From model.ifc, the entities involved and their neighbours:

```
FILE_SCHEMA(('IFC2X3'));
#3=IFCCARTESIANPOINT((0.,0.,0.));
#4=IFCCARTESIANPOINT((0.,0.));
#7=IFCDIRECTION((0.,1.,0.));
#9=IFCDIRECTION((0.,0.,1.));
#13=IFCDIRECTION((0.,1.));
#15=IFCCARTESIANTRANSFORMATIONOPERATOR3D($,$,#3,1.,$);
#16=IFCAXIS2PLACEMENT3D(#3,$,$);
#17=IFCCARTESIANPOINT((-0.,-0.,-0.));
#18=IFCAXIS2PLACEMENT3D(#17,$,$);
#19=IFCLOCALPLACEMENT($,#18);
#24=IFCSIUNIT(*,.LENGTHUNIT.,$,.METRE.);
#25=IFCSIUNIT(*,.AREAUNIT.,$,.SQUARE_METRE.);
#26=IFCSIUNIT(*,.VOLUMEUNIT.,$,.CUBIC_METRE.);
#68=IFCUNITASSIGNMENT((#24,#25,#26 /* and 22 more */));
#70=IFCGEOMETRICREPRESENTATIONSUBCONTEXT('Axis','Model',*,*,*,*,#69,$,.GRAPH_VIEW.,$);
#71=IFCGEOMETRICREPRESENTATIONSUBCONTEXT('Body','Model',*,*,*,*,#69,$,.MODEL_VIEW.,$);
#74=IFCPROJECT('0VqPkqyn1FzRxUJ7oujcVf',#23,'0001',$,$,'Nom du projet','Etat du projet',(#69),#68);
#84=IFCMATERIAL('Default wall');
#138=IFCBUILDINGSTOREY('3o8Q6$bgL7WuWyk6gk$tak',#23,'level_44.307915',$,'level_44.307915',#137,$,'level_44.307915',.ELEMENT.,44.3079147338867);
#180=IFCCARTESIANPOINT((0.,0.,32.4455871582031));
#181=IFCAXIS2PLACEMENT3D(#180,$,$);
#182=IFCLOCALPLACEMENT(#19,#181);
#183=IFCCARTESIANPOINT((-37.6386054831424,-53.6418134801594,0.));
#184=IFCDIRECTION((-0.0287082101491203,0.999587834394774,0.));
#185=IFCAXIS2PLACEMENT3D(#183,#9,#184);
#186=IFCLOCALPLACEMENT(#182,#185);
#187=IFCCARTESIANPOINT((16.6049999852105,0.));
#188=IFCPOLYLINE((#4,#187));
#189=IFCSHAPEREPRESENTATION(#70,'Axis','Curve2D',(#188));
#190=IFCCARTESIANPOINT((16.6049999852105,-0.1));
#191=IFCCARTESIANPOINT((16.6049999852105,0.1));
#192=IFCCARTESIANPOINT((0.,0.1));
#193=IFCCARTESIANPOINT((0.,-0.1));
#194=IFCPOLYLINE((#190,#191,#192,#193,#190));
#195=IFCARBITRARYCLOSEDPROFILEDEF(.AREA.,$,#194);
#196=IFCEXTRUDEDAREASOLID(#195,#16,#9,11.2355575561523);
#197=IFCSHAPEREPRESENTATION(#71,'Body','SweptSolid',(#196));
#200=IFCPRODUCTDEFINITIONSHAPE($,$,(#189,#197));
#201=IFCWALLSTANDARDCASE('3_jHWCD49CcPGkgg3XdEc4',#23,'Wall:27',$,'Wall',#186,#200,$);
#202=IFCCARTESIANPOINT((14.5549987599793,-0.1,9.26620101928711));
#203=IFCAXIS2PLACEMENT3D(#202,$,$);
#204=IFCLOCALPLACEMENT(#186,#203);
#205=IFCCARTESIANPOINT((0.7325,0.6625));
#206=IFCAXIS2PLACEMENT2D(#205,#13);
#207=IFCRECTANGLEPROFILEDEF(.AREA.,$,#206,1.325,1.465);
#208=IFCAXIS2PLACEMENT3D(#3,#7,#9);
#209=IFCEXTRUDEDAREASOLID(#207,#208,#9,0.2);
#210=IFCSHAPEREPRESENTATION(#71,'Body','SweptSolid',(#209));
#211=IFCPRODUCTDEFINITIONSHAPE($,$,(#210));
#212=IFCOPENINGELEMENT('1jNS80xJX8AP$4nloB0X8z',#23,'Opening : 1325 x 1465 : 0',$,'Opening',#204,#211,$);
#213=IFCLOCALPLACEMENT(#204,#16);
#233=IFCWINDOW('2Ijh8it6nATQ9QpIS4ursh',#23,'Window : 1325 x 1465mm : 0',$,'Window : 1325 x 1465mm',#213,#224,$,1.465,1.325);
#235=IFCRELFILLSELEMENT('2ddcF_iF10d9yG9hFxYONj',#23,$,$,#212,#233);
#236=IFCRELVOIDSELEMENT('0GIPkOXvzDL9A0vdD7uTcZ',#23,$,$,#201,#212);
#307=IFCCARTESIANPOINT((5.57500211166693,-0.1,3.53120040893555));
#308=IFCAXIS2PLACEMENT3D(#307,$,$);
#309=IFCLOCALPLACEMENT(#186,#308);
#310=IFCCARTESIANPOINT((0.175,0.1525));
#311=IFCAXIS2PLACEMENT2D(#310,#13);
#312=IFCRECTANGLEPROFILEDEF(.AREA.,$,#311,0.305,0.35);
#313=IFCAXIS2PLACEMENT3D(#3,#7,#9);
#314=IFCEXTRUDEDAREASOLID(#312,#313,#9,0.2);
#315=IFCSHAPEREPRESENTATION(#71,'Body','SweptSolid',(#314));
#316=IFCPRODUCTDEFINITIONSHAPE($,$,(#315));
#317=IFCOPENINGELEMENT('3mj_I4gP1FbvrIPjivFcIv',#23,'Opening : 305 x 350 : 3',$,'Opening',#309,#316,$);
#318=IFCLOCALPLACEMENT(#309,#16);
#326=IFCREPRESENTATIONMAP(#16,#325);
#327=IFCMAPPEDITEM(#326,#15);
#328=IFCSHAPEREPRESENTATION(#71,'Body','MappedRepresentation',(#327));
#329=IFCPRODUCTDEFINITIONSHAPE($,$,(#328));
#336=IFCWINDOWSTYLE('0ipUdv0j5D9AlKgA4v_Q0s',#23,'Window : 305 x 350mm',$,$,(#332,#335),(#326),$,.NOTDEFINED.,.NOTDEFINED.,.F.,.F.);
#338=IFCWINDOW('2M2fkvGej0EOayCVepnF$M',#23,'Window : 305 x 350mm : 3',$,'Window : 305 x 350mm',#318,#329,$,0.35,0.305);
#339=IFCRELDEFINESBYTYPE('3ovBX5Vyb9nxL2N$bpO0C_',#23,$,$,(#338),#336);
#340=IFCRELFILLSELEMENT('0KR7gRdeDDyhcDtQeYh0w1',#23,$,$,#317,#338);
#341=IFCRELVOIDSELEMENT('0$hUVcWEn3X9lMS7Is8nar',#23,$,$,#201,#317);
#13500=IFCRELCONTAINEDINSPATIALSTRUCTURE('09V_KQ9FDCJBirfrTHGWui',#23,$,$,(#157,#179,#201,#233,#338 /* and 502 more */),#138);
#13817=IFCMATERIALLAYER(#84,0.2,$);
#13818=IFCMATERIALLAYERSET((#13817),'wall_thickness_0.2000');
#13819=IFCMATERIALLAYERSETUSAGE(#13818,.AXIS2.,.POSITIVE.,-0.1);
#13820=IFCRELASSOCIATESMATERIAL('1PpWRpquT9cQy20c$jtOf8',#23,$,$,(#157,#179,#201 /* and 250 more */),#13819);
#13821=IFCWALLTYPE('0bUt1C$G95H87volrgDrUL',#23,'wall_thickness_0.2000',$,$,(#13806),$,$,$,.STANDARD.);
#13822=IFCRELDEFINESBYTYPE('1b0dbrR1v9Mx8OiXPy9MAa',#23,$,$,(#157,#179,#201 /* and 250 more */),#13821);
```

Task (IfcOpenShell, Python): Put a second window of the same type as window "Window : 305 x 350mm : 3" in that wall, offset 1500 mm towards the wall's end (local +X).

```python
import ifcopenshell
import ifcopenshell.api.feature
import ifcopenshell.api.geometry
import ifcopenshell.api.root
import ifcopenshell.geom
import ifcopenshell.util.element
import ifcopenshell.util.placement
import ifcopenshell.util.shape
import ifcopenshell.util.unit

model = ifcopenshell.open("model.ifc")
unit_scale = ifcopenshell.util.unit.calculate_unit_scale(model)
settings = ifcopenshell.geom.settings()


def volume(element):
    """Net volume in cubic metres, openings subtracted."""
    shape = ifcopenshell.geom.create_shape(settings, element)
    return ifcopenshell.util.shape.get_volume(shape.geometry)


window = model.by_guid("2M2fkvGej0EOayCVepnF$M")
opening = window.FillsVoids[0].RelatingOpeningElement
wall = opening.VoidsElements[0].RelatingBuildingElement
before = volume(wall)
shift = ifcopenshell.util.placement.get_local_placement(wall.ObjectPlacement)[:3, 0] * 1.5 / unit_scale

# copy_class copies the void relationship, type, container and properties, but no geometry.
new_opening = ifcopenshell.api.root.copy_class(model, product=opening)
new_opening.Representation = ifcopenshell.util.element.copy_deep(
    model, opening.Representation, exclude=["IfcGeometricRepresentationContext", "IfcRepresentationMap"]
)
new_opening.Name = "Opening : 305 x 350"
new_window = ifcopenshell.api.root.copy_class(model, product=window)
new_window.Representation = ifcopenshell.util.element.copy_deep(
    model, window.Representation, exclude=["IfcGeometricRepresentationContext", "IfcRepresentationMap"]
)
new_window.Name = "Window : 305 x 350mm"
fills = ifcopenshell.api.feature.add_filling(model, opening=new_opening, element=new_window)
fills.OwnerHistory = new_window.OwnerHistory  # required in IFC2X3

for old, new in ((opening, new_opening), (window, new_window)):
    matrix = ifcopenshell.util.placement.get_local_placement(old.ObjectPlacement)
    matrix[:3, 3] += shift
    ifcopenshell.api.geometry.edit_object_placement(model, product=new, matrix=matrix, is_si=False)

after = volume(wall)

print(f"wall volume {before:.3f} -> {after:.3f} m3")

model.write("model_rev.ifc")
```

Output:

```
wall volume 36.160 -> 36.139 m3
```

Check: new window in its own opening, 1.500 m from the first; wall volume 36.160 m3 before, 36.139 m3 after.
